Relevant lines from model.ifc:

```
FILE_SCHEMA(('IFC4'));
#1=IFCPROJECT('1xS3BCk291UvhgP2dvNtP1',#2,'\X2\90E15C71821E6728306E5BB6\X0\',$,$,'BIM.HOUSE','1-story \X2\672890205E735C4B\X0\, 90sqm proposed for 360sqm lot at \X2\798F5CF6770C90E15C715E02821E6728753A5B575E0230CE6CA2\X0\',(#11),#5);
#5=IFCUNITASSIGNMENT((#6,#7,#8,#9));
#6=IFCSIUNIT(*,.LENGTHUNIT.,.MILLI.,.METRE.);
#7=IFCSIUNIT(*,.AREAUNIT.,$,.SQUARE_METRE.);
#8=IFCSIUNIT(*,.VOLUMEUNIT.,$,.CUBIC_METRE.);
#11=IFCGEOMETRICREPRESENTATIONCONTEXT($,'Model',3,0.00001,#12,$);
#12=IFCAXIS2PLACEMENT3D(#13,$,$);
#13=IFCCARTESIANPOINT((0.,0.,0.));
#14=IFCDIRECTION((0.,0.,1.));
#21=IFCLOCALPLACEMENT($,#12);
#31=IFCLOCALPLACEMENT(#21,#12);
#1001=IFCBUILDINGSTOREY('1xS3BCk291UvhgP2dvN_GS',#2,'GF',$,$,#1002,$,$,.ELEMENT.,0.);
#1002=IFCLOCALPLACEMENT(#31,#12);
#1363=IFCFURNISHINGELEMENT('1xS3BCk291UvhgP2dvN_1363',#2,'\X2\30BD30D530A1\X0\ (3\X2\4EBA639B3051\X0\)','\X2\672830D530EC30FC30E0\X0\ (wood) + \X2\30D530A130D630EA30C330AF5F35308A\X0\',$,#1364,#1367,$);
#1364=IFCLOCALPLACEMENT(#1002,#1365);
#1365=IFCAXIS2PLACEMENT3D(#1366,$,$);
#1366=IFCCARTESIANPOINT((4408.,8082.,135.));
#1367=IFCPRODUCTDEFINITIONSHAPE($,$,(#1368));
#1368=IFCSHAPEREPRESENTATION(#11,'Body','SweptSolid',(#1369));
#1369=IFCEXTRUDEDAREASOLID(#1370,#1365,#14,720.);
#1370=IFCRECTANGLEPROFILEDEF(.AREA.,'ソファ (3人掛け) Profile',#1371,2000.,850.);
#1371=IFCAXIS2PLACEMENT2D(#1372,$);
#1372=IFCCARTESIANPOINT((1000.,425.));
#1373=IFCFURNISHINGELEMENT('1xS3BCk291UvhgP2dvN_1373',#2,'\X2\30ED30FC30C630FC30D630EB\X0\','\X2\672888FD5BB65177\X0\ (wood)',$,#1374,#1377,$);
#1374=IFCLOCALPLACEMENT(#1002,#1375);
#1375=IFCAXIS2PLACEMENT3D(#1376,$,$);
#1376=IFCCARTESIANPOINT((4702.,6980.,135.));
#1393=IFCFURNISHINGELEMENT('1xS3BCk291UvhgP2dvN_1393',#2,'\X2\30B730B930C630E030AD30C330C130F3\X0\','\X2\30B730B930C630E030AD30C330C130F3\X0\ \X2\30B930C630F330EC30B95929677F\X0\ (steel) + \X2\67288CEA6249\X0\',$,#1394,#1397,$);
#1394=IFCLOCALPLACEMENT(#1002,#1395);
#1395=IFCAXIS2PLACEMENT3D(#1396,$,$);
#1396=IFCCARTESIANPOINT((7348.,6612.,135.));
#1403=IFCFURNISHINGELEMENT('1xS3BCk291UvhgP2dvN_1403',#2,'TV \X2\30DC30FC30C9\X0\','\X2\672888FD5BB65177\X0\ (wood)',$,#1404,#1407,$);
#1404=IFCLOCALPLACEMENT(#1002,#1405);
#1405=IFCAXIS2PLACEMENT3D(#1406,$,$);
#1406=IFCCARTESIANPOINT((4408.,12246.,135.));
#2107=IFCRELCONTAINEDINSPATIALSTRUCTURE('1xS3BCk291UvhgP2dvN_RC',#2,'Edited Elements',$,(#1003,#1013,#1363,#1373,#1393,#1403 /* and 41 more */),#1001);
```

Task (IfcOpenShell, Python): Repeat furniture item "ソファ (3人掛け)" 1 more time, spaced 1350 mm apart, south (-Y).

```python
import numpy as np
import ifcopenshell
import ifcopenshell.api.geometry
import ifcopenshell.api.root
import ifcopenshell.util.element
import ifcopenshell.util.placement

model = ifcopenshell.open("model.ifc")


def reuse_history(source, copy):
    """copy_class also copies each property set's owner history, people and application; keep the originals."""
    for rel in copy.IsDefinedBy:
        if rel.is_a("IfcRelDefinesByProperties") and (history := rel.RelatingPropertyDefinition.OwnerHistory):
            rel.RelatingPropertyDefinition.OwnerHistory = source.OwnerHistory
            ifcopenshell.util.element.remove_deep2(model, history)


source = model.by_guid("1xS3BCk291UvhgP2dvN_1363")
base = ifcopenshell.util.placement.get_local_placement(source.ObjectPlacement)
step = np.array([0.0, -1.0, 0.0]) * 1350.0

for i in range(1, 2):
    copy = ifcopenshell.api.root.copy_class(model, product=source)
    copy.Representation = ifcopenshell.util.element.copy_deep(
        model, source.Representation, exclude=["IfcGeometricRepresentationContext", "IfcRepresentationMap"]
    )
    reuse_history(source, copy)
    matrix = base.copy()
    matrix[:3, 3] += i * step
    print("added at", matrix[:3, 3].round(3) + 0.0)
    ifcopenshell.api.geometry.edit_object_placement(model, product=copy, matrix=matrix, is_si=False)

model.write("model-out.ifc")
```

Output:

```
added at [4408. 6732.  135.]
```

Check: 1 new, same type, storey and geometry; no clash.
